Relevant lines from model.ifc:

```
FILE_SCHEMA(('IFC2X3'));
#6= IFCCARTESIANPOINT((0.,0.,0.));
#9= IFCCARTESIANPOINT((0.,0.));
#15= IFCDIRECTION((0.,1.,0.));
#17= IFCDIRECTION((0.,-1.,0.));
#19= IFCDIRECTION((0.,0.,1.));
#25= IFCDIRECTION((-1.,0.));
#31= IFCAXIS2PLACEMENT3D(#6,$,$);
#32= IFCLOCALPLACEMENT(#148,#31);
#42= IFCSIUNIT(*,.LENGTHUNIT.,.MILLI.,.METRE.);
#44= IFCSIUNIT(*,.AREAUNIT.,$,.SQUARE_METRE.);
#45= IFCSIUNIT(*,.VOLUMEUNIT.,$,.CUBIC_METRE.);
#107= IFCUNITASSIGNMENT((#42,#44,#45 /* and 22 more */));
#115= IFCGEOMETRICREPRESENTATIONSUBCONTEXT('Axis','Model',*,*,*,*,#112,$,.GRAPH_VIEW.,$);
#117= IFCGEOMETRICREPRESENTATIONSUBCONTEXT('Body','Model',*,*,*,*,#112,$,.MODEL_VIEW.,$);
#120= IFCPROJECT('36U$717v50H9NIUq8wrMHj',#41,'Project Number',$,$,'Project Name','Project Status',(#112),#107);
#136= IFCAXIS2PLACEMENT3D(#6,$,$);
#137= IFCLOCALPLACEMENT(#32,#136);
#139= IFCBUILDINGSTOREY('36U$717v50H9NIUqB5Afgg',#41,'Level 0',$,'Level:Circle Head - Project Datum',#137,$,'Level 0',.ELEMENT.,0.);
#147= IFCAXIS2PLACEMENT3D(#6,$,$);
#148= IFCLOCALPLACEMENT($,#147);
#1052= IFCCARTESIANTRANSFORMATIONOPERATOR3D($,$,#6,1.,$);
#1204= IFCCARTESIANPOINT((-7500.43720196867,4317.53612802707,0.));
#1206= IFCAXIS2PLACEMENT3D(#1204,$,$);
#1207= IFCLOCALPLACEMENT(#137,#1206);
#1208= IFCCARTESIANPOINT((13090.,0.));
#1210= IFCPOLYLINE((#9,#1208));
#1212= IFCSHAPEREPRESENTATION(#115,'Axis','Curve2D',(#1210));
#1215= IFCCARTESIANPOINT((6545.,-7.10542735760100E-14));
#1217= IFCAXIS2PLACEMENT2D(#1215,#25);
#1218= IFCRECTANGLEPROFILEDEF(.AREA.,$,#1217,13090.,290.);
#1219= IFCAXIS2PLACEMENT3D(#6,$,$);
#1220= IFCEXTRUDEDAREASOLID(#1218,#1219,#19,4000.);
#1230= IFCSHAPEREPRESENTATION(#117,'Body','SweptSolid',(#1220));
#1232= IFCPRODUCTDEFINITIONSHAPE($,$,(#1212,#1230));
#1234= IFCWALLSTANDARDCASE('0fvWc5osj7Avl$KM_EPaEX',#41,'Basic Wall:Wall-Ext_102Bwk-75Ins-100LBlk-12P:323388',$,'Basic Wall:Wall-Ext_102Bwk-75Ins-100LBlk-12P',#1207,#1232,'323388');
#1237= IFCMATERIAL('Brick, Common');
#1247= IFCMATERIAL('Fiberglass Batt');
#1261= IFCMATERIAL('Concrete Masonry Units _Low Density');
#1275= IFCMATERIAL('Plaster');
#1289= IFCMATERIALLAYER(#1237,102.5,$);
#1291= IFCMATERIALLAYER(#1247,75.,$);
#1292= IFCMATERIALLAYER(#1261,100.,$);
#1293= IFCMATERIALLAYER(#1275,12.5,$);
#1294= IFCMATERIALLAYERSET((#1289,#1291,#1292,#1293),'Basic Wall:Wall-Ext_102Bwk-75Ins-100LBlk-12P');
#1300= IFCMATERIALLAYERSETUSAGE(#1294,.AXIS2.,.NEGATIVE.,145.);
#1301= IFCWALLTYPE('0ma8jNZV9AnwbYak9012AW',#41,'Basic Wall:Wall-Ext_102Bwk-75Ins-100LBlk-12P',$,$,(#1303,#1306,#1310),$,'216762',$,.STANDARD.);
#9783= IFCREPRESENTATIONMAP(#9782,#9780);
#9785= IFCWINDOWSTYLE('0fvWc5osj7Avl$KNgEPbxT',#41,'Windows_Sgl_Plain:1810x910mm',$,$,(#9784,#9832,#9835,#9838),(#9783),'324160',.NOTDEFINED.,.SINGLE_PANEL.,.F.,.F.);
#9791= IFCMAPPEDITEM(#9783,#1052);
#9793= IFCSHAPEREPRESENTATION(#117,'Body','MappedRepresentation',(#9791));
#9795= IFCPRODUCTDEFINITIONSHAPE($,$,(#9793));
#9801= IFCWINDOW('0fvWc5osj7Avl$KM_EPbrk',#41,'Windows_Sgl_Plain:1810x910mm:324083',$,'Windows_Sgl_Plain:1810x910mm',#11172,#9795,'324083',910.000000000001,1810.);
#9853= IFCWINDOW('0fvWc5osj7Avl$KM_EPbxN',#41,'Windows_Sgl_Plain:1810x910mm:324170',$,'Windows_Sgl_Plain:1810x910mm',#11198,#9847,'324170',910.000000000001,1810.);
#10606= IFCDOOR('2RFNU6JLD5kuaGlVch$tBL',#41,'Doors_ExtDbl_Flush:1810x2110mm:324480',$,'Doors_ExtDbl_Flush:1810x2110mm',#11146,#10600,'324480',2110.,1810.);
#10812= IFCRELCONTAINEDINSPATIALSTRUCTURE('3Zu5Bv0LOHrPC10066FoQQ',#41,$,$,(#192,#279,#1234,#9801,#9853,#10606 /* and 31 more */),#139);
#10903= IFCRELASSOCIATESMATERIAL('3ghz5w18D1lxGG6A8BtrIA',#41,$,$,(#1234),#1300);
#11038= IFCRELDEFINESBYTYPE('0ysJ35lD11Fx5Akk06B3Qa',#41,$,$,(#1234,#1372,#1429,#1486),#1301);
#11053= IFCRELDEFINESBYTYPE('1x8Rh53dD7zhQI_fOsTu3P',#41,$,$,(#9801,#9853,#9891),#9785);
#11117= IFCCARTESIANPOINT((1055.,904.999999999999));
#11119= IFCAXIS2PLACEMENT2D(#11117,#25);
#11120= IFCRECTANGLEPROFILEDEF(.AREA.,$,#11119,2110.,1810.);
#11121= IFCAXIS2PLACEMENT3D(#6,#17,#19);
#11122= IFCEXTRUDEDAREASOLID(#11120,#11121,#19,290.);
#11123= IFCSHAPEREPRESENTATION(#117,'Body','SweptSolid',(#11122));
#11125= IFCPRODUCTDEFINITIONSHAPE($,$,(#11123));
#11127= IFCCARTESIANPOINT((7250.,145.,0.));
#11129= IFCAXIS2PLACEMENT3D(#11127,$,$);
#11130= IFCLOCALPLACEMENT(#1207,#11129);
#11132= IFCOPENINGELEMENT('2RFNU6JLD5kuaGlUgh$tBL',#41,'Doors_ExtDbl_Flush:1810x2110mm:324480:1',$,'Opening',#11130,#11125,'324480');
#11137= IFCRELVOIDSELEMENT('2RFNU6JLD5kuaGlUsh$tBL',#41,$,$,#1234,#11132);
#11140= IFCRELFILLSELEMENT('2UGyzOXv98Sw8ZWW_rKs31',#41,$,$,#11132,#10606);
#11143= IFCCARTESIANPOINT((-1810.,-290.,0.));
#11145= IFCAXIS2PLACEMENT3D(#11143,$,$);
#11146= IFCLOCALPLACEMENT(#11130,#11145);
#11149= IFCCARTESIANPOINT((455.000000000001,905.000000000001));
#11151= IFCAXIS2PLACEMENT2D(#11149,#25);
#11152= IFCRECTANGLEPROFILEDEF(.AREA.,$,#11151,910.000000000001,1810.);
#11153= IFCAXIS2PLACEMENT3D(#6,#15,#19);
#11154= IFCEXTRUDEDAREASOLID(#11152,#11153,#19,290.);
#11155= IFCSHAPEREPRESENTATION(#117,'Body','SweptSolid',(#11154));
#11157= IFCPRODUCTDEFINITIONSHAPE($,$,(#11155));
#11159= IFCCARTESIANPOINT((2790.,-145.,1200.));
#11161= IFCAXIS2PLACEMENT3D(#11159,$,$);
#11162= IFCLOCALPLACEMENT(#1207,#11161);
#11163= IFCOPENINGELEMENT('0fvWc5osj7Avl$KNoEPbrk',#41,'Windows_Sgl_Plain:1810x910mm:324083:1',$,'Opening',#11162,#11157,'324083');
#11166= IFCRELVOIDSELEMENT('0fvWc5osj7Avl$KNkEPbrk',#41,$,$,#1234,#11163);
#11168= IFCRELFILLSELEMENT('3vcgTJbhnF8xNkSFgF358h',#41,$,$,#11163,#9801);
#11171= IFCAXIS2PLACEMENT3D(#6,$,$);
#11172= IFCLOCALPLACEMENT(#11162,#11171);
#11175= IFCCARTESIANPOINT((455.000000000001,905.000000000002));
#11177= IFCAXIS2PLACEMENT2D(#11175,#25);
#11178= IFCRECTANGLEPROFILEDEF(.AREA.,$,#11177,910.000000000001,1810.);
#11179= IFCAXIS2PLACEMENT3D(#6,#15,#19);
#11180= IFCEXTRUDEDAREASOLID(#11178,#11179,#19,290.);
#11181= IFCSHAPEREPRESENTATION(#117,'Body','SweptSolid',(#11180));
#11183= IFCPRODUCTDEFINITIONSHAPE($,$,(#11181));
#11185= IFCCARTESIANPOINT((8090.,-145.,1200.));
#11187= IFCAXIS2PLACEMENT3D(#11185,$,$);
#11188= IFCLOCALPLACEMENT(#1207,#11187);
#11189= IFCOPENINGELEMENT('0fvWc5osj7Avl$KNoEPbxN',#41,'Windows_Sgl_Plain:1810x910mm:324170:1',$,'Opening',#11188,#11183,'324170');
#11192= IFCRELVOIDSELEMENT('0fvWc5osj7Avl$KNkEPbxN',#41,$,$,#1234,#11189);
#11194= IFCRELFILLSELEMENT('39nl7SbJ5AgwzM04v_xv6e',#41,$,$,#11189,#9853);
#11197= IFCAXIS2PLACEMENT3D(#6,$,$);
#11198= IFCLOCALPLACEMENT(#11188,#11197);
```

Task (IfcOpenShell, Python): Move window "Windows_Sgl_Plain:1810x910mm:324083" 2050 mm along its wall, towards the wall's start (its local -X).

```python
import ifcopenshell
import ifcopenshell.api.geometry
import ifcopenshell.util.placement
import ifcopenshell.util.unit

model = ifcopenshell.open("model.ifc")
unit_scale = ifcopenshell.util.unit.calculate_unit_scale(model)

window = model.by_guid("0fvWc5osj7Avl$KM_EPbrk")
opening = window.FillsVoids[0].RelatingOpeningElement
wall = opening.VoidsElements[0].RelatingBuildingElement

wall_matrix = ifcopenshell.util.placement.get_local_placement(wall.ObjectPlacement)
shift = wall_matrix[:3, 0] * -2.05 / unit_scale
before = ifcopenshell.util.placement.get_local_placement(window.ObjectPlacement)[:3, 3].copy()

# The window is placed relative to its opening, so it follows when the opening moves.
matrix = ifcopenshell.util.placement.get_local_placement(opening.ObjectPlacement)
matrix[:3, 3] += shift
ifcopenshell.api.geometry.edit_object_placement(
    model, product=opening, matrix=matrix, is_si=False, should_transform_children=True
)

after = ifcopenshell.util.placement.get_local_placement(window.ObjectPlacement)[:3, 3]
print("window moved by", (after - before).round(3) + 0.0)

model.write("model_edited.ifc")
```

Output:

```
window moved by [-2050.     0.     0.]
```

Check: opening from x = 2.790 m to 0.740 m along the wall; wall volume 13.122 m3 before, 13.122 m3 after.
